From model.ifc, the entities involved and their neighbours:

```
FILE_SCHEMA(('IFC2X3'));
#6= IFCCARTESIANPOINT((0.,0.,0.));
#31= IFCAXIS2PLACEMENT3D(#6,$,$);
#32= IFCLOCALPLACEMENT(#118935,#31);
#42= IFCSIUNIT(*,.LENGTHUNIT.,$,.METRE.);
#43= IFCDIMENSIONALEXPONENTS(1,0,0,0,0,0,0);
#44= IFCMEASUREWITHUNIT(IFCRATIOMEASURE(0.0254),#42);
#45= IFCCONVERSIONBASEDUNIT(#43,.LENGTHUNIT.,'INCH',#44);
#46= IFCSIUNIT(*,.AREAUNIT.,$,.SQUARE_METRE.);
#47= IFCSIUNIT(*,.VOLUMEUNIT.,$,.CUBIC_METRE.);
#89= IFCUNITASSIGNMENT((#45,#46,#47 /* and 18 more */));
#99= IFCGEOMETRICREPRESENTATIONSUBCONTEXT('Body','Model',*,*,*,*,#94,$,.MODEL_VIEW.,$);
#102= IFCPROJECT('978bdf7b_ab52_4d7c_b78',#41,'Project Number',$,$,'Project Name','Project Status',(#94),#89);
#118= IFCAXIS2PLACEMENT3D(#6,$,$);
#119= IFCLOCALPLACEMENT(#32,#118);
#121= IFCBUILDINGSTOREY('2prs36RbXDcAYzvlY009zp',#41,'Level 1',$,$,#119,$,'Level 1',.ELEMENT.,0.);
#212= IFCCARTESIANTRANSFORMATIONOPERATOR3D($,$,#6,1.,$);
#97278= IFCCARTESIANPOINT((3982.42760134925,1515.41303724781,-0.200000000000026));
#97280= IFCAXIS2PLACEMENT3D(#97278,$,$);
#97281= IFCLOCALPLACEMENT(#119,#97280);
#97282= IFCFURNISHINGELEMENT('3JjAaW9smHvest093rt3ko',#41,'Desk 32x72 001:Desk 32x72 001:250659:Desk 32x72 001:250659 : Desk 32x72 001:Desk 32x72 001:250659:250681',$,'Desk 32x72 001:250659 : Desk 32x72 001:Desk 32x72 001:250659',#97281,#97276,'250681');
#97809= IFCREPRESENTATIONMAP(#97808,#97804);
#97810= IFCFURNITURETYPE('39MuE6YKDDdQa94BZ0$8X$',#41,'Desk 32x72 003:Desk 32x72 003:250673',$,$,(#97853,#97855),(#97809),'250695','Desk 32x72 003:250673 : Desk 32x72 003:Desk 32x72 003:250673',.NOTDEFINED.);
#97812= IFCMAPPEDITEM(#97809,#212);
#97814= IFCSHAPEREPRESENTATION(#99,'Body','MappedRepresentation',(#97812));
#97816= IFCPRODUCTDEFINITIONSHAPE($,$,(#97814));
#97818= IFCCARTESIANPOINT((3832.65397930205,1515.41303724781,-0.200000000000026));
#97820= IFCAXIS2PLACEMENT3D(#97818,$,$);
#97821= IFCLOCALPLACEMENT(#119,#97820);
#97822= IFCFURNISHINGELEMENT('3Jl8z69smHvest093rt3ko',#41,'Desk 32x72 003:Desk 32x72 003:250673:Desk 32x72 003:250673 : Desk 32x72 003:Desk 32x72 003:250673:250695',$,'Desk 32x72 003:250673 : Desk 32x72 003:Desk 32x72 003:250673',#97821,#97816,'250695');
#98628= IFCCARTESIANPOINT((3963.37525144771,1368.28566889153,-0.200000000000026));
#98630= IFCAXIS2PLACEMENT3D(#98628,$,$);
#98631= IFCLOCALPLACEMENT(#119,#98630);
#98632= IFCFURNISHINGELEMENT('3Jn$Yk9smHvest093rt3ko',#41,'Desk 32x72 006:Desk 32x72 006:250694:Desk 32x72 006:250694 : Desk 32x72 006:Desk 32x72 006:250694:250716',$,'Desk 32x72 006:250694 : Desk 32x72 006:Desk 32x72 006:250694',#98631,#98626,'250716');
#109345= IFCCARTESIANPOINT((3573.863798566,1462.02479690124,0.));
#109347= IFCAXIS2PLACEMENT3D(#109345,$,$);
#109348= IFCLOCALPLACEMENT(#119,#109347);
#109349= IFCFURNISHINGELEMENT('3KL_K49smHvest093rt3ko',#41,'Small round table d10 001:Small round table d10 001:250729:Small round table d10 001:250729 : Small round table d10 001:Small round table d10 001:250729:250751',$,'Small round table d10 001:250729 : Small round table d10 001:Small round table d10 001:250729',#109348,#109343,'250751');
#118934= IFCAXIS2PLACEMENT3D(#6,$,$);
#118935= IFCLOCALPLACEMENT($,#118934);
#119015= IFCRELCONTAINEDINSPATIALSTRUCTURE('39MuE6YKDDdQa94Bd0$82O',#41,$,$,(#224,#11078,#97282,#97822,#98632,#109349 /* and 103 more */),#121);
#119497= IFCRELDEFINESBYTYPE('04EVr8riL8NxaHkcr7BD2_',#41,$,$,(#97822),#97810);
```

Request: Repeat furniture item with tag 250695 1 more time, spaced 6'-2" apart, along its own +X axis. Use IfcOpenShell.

```python
import ifcopenshell
import ifcopenshell.api.geometry
import ifcopenshell.api.root
import ifcopenshell.util.element
import ifcopenshell.util.placement
import ifcopenshell.util.unit

model = ifcopenshell.open("model.ifc")
unit_scale = ifcopenshell.util.unit.calculate_unit_scale(model)


def reuse_history(source, copy):
    """copy_class also copies each property set's owner history, people and application; keep the originals."""
    for rel in copy.IsDefinedBy:
        if rel.is_a("IfcRelDefinesByProperties") and (history := rel.RelatingPropertyDefinition.OwnerHistory):
            rel.RelatingPropertyDefinition.OwnerHistory = source.OwnerHistory
            ifcopenshell.util.element.remove_deep2(model, history)


source = model.by_id(97822)
base = ifcopenshell.util.placement.get_local_placement(source.ObjectPlacement)
step = base[:3, 0] * 74 * 0.0254 / unit_scale

for i in range(1, 2):
    copy = ifcopenshell.api.root.copy_class(model, product=source)
    copy.Representation = ifcopenshell.util.element.copy_deep(
        model, source.Representation, exclude=["IfcGeometricRepresentationContext", "IfcRepresentationMap"]
    )
    copy.Name = "Desk 32x72 003:Desk 32x72 003:250673:Desk 32x72 003:250673 : Desk 32x72 003:Desk 32x72 003"
    copy.Tag = None
    reuse_history(source, copy)
    matrix = base.copy()
    matrix[:3, 3] += i * step
    print("added at", matrix[:3, 3].round(3) + 0.0)
    ifcopenshell.api.geometry.edit_object_placement(model, product=copy, matrix=matrix, is_si=False)

model.write("model_v2.ifc")
```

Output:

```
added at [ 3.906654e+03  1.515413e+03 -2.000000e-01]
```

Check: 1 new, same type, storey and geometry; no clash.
